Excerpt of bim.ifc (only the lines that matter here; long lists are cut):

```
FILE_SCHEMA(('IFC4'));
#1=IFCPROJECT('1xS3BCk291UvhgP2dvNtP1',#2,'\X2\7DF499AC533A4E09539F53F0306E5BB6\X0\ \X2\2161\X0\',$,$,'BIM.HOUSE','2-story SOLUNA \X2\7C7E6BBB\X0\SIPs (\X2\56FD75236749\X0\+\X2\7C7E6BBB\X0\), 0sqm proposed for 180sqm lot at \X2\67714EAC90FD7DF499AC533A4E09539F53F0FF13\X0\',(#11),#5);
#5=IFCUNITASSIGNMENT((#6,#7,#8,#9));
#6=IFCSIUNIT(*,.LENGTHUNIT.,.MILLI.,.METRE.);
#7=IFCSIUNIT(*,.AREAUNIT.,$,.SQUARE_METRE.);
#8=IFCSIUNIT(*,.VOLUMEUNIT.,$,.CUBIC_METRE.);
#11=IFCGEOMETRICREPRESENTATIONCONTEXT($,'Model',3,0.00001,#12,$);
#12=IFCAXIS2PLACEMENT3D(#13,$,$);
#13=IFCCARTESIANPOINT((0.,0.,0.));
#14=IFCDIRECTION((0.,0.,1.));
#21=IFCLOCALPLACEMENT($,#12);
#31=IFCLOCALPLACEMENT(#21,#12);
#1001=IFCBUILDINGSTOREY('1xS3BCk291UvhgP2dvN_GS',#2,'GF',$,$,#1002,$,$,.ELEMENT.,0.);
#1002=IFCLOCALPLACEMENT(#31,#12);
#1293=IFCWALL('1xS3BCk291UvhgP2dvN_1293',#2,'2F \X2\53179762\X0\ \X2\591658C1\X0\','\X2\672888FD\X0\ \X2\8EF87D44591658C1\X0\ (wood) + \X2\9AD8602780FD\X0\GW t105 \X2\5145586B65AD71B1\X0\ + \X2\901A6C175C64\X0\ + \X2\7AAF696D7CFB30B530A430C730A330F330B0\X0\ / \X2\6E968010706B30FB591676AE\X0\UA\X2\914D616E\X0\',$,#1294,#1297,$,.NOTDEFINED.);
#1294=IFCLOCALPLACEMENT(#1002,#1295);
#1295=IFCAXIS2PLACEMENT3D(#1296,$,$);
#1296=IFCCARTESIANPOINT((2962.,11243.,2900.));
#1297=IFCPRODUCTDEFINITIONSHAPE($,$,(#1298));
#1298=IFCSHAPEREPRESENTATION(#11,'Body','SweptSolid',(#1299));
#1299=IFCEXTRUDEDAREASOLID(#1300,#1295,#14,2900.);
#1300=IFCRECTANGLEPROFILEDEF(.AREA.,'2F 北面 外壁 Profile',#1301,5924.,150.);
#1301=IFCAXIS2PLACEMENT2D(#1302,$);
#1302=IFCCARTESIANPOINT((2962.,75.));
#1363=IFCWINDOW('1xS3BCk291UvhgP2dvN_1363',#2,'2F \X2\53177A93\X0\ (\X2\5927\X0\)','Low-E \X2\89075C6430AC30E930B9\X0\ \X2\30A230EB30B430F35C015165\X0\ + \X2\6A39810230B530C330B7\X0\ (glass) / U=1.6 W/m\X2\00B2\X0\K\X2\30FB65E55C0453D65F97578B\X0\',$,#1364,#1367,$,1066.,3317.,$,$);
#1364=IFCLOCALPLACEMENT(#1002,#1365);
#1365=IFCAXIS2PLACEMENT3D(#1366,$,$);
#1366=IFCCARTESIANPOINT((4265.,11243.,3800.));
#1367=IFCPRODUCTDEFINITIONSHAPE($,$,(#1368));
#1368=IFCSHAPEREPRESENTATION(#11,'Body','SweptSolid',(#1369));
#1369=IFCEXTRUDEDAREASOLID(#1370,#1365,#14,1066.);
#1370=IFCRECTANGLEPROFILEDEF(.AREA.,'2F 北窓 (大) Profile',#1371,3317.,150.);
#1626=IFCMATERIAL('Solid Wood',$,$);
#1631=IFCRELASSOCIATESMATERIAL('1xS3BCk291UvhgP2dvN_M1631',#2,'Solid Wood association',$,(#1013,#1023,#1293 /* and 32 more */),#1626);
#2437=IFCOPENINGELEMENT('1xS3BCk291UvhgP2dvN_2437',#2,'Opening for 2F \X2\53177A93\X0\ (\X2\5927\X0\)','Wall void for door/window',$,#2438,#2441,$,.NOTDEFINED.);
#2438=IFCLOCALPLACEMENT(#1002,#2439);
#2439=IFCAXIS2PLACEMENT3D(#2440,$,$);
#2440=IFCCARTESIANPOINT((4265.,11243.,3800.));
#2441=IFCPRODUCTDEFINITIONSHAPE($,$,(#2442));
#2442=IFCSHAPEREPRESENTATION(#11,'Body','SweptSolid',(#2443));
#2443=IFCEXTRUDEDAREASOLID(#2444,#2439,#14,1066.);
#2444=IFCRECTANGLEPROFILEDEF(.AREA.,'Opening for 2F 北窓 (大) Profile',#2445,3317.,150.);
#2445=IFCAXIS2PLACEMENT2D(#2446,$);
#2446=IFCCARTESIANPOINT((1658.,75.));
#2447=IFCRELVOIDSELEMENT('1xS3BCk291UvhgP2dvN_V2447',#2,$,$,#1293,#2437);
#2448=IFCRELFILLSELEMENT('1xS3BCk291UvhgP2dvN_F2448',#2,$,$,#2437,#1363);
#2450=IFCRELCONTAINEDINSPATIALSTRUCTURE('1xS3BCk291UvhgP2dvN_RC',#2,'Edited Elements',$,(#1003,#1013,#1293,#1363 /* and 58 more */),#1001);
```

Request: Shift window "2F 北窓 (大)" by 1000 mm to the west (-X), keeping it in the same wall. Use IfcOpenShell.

```python
import ifcopenshell
import ifcopenshell.api.geometry
import ifcopenshell.util.placement

model = ifcopenshell.open("bim.ifc")

window = model.by_id(1363)
opening = window.FillsVoids[0].RelatingOpeningElement
wall = opening.VoidsElements[0].RelatingBuildingElement

wall_matrix = ifcopenshell.util.placement.get_local_placement(wall.ObjectPlacement)
shift = wall_matrix[:3, 0] * -1000.0
before = ifcopenshell.util.placement.get_local_placement(window.ObjectPlacement)[:3, 3].copy()

# The window is not placed relative to its opening, so move both.
for product in (opening, window):
    matrix = ifcopenshell.util.placement.get_local_placement(product.ObjectPlacement)
    matrix[:3, 3] += shift
    ifcopenshell.api.geometry.edit_object_placement(model, product=product, matrix=matrix, is_si=False)

after = ifcopenshell.util.placement.get_local_placement(window.ObjectPlacement)[:3, 3]
print("window moved by", (after - before).round(3) + 0.0)

model.write("bim_edited.ifc")
```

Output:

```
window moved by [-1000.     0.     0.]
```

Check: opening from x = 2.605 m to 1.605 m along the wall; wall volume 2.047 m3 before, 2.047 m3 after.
